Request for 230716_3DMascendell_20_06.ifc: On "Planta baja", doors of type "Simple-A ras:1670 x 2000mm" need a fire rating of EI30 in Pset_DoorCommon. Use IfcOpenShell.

First a look at what the model holds.

```python
import ifcopenshell
import ifcopenshell.util.element

model = ifcopenshell.open("230716_3DMascendell_20_06.ifc")
print(model.schema)
storey = next(s for s in model.by_type("IfcBuildingStorey") if s.Name == "Planta baja")
doors = [e for e in ifcopenshell.util.element.get_decomposition(storey) if e.is_a("IfcDoor")]
seen = {}
for e in doors:
    element_type = ifcopenshell.util.element.get_type(e)
    key = (element_type.Name if element_type != e and element_type else None, ifcopenshell.util.element.get_pset(e, "Pset_DoorCommon", "FireRating"))
    seen[key] = seen.get(key, 0) + 1
for (name, value), count in sorted(seen.items(), key=str):
    print(count, "x", name, "|", value)
```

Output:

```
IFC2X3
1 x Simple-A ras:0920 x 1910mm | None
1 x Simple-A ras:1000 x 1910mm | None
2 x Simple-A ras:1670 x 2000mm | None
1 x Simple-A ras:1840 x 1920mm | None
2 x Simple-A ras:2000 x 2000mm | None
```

```python
import ifcopenshell
import ifcopenshell.api.pset
import ifcopenshell.util.element

model = ifcopenshell.open("230716_3DMascendell_20_06.ifc")

storey = next(s for s in model.by_type("IfcBuildingStorey") if s.Name == "Planta baja")
doors = [e for e in ifcopenshell.util.element.get_decomposition(storey) if e.is_a("IfcDoor")]

count = 0
for e in doors:
    element_type = ifcopenshell.util.element.get_type(e)
    if element_type in (None, e) or element_type.Name != "Simple-A ras:1670 x 2000mm":
        continue
    # add_pset returns the element's existing set when there is one.
    pset = ifcopenshell.api.pset.add_pset(model, product=e, name="Pset_DoorCommon")
    ifcopenshell.api.pset.edit_pset(model, pset=pset, properties={"FireRating": "EI30"})
    count += 1

print(count, "doors updated")

model.write("230716_3DMascendell_20_06-out.ifc")
```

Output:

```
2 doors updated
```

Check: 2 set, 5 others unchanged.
